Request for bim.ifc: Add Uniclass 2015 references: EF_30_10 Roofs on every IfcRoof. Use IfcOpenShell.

First a look at what the model holds.

```python
import ifcopenshell

model = ifcopenshell.open("bim.ifc")
print(model.schema)
print("classifications:", [c.Name for c in model.by_type("IfcClassification")])
for ifc_class in ("IfcDoor", "IfcRoof", "IfcStair", "IfcWall", "IfcWindow"):
    print(ifc_class, len(model.by_type(ifc_class)))
```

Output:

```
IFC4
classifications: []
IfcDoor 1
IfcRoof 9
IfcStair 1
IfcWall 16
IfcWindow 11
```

```python
import ifcopenshell
import ifcopenshell.api.classification

model = ifcopenshell.open("bim.ifc")

system = ifcopenshell.api.classification.add_classification(model, classification="Uniclass 2015")

codes = {
    "IfcRoof": ("EF_30_10", "Roofs"),
}
for ifc_class, (code, name) in codes.items():
    products = model.by_type(ifc_class)
    ifcopenshell.api.classification.add_reference(
        model, products=products, classification=system, identification=code, name=name
    )
    print(code, len(products))

model.write("bim_rev.ifc")
```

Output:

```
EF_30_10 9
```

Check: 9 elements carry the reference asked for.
